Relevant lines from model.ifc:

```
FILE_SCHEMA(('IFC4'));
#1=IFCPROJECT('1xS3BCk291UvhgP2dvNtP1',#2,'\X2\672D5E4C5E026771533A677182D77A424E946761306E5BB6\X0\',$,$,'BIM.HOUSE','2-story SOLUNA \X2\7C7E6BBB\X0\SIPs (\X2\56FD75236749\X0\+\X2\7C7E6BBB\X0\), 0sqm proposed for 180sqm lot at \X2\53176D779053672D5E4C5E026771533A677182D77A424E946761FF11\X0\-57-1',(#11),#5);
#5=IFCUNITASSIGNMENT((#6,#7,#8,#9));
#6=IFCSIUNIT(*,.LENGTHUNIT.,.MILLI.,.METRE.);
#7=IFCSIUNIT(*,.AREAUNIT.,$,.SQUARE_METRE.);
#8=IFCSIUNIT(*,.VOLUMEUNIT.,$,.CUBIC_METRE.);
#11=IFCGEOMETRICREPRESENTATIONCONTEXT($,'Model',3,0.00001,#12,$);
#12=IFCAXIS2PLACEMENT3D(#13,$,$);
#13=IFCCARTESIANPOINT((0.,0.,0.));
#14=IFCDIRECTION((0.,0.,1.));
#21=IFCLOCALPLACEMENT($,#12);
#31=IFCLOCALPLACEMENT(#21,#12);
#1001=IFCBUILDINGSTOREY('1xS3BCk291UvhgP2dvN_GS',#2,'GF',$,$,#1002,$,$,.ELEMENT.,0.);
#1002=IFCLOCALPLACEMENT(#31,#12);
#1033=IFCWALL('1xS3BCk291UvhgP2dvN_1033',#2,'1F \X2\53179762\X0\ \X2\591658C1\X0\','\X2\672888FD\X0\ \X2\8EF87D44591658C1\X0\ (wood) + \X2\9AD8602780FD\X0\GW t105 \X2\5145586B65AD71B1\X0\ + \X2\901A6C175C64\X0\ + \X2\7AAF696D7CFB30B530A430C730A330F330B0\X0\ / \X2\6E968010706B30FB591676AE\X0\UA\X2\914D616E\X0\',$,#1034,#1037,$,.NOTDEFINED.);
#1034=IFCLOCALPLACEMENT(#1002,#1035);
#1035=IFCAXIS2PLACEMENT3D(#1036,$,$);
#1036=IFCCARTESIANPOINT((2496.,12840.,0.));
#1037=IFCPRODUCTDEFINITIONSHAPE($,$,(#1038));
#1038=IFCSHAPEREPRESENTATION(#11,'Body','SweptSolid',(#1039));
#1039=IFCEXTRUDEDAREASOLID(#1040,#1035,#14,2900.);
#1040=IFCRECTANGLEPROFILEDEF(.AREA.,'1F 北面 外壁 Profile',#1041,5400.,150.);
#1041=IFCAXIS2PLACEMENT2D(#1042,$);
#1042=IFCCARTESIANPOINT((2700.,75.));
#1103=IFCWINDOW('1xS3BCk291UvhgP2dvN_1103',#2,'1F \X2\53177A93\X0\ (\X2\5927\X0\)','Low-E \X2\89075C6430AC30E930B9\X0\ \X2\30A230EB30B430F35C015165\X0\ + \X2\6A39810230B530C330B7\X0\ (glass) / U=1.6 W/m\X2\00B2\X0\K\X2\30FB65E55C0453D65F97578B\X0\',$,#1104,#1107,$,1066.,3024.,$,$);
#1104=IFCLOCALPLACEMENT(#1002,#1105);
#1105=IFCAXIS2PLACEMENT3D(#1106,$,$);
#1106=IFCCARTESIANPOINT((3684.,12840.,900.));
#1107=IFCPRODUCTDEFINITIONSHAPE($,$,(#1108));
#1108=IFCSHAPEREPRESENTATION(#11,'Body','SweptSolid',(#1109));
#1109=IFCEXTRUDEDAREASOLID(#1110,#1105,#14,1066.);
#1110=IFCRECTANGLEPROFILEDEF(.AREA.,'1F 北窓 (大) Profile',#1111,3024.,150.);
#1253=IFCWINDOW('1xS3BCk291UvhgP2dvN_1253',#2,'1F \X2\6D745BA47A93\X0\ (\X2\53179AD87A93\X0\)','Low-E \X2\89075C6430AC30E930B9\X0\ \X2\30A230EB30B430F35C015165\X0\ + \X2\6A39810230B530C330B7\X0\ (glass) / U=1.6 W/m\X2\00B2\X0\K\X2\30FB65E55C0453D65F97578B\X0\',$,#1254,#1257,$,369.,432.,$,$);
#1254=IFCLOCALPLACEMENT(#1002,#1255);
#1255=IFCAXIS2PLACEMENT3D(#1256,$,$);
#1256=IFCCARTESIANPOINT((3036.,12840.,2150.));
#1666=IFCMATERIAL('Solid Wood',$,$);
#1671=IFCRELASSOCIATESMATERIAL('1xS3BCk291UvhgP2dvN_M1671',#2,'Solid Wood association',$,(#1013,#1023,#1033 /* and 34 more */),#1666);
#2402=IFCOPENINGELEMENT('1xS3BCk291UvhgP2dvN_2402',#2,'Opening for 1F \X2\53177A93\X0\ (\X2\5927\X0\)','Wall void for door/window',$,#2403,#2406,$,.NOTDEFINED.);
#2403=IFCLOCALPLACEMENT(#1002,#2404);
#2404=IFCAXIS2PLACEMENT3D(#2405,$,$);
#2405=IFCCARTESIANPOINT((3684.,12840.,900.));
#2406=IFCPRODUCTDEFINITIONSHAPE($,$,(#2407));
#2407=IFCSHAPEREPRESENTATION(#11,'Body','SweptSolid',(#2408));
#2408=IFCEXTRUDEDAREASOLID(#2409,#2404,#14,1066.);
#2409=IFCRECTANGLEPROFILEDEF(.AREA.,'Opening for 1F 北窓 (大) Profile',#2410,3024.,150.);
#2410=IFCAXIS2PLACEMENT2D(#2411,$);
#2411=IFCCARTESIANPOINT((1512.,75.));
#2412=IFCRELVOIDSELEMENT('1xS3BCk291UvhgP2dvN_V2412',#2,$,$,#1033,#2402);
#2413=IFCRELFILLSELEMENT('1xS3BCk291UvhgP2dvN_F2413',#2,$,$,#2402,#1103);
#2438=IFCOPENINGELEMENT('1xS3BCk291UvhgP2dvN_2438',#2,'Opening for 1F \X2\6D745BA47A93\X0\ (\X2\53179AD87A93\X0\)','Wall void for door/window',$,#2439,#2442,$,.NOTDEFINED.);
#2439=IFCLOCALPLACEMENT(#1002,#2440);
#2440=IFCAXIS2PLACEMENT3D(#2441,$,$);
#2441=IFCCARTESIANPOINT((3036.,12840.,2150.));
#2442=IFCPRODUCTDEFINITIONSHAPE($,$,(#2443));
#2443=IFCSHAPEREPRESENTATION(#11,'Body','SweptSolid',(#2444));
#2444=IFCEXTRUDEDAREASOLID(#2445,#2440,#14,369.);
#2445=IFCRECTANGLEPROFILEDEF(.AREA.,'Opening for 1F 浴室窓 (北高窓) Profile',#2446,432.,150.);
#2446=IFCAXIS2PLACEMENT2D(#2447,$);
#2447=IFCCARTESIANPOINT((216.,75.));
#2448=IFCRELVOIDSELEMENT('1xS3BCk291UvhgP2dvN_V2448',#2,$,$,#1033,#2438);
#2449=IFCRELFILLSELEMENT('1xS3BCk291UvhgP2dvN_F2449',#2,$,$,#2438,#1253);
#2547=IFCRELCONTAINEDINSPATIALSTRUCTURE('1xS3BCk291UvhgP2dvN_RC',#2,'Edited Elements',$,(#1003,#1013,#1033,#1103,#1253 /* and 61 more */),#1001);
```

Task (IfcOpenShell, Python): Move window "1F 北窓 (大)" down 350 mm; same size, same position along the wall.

```python
import numpy as np
import ifcopenshell
import ifcopenshell.api.geometry
import ifcopenshell.util.placement
import ifcopenshell.util.unit

model = ifcopenshell.open("model.ifc")
unit_scale = ifcopenshell.util.unit.calculate_unit_scale(model)

window = model.by_guid("1xS3BCk291UvhgP2dvN_1103")
opening = window.FillsVoids[0].RelatingOpeningElement
dz = -0.35 / unit_scale

shift = np.array([0.0, 0.0, dz])
# The window is not placed relative to its opening, so move both.
for product in (opening, window):
    matrix = ifcopenshell.util.placement.get_local_placement(product.ObjectPlacement)
    matrix[:3, 3] += shift
    ifcopenshell.api.geometry.edit_object_placement(model, product=product, matrix=matrix, is_si=False)

print(f"moved by {dz * unit_scale:+.3f} m")

model.write("model_updated.ifc")
```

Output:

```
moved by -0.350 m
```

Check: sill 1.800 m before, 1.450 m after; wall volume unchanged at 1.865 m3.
